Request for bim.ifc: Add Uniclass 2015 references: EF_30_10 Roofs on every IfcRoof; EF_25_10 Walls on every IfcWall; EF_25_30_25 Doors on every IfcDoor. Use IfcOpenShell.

First a look at what the model holds.

```python
import ifcopenshell

model = ifcopenshell.open("bim.ifc")
print(model.schema)
print("classifications:", [c.Name for c in model.by_type("IfcClassification")])
for ifc_class in ("IfcDoor", "IfcRoof", "IfcStair", "IfcWall", "IfcWindow"):
    print(ifc_class, len(model.by_type(ifc_class)))
```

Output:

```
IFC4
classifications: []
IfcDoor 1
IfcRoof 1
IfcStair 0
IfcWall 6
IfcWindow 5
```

```python
import ifcopenshell
import ifcopenshell.api.classification

model = ifcopenshell.open("bim.ifc")

system = ifcopenshell.api.classification.add_classification(model, classification="Uniclass 2015")

codes = {
    "IfcRoof": ("EF_30_10", "Roofs"),
    "IfcWall": ("EF_25_10", "Walls"),
    "IfcDoor": ("EF_25_30_25", "Doors"),
}
for ifc_class, (code, name) in codes.items():
    products = model.by_type(ifc_class)
    ifcopenshell.api.classification.add_reference(
        model, products=products, classification=system, identification=code, name=name
    )
    print(code, len(products))

model.write("bim-out.ifc")
```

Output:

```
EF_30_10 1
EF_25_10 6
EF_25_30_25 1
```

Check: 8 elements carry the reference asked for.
